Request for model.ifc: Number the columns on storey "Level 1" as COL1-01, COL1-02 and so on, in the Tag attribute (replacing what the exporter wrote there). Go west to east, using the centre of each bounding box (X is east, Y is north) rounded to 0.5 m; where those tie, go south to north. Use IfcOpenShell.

First a look at what the model holds.

```python
import ifcopenshell
import ifcopenshell.util.element
import ifcopenshell.util.placement

model = ifcopenshell.open("model.ifc")
print(model.schema)
storey = next(s for s in model.by_type("IfcBuildingStorey") if s.Name == "Level 1")
columns = [e for e in ifcopenshell.util.element.get_decomposition(storey) if e.is_a("IfcColumn")]
for e in sorted(columns, key=lambda e: e.id()):
    origin = ifcopenshell.util.placement.get_local_placement(e.ObjectPlacement)[:3, 3]
    print(e.id(), e.Tag, e.Name, origin.round(2) + 0.0, sep=" | ")
```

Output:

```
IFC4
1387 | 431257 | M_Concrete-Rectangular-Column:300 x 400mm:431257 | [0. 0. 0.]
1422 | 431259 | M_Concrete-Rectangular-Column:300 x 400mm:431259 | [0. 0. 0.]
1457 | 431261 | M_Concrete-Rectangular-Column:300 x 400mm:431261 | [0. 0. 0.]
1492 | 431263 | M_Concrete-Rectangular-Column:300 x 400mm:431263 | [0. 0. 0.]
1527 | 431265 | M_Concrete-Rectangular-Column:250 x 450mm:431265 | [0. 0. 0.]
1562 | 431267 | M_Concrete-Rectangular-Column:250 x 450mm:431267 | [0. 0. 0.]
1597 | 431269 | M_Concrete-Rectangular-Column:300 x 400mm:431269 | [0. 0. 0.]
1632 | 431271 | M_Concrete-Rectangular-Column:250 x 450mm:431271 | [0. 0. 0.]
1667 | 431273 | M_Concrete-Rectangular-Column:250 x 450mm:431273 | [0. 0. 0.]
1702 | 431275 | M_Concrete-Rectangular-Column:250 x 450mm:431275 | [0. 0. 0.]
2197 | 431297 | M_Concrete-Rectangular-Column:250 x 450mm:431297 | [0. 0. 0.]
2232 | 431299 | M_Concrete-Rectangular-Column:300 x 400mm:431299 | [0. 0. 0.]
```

```python
import ifcopenshell
import ifcopenshell.geom
import ifcopenshell.util.element
import ifcopenshell.util.shape

model = ifcopenshell.open("model.ifc")
settings = ifcopenshell.geom.settings()
settings.set("use-world-coords", True)


def centre(element):
    shape = ifcopenshell.geom.create_shape(settings, element)
    return ifcopenshell.util.shape.get_bbox_centroid(shape.geometry)


storey = next(s for s in model.by_type("IfcBuildingStorey") if s.Name == "Level 1")
columns = [e for e in ifcopenshell.util.element.get_decomposition(storey) if e.is_a("IfcColumn")]

# Insertion points can sit at a corner or the storey origin, so sort by the geometry (in metres).
centres = {e: centre(e) for e in columns}
columns.sort(key=lambda e: (round(centres[e][0] / 0.5), centres[e][1]))

for i, e in enumerate(columns, start=1):
    number = f"COL1-{i:02d}"
    e.Tag = number
    print(e.id(), number)

model.write("model-out.ifc")
```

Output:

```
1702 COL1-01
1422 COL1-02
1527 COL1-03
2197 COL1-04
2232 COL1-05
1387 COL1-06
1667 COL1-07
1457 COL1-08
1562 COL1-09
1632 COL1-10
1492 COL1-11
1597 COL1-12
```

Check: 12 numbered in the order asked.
